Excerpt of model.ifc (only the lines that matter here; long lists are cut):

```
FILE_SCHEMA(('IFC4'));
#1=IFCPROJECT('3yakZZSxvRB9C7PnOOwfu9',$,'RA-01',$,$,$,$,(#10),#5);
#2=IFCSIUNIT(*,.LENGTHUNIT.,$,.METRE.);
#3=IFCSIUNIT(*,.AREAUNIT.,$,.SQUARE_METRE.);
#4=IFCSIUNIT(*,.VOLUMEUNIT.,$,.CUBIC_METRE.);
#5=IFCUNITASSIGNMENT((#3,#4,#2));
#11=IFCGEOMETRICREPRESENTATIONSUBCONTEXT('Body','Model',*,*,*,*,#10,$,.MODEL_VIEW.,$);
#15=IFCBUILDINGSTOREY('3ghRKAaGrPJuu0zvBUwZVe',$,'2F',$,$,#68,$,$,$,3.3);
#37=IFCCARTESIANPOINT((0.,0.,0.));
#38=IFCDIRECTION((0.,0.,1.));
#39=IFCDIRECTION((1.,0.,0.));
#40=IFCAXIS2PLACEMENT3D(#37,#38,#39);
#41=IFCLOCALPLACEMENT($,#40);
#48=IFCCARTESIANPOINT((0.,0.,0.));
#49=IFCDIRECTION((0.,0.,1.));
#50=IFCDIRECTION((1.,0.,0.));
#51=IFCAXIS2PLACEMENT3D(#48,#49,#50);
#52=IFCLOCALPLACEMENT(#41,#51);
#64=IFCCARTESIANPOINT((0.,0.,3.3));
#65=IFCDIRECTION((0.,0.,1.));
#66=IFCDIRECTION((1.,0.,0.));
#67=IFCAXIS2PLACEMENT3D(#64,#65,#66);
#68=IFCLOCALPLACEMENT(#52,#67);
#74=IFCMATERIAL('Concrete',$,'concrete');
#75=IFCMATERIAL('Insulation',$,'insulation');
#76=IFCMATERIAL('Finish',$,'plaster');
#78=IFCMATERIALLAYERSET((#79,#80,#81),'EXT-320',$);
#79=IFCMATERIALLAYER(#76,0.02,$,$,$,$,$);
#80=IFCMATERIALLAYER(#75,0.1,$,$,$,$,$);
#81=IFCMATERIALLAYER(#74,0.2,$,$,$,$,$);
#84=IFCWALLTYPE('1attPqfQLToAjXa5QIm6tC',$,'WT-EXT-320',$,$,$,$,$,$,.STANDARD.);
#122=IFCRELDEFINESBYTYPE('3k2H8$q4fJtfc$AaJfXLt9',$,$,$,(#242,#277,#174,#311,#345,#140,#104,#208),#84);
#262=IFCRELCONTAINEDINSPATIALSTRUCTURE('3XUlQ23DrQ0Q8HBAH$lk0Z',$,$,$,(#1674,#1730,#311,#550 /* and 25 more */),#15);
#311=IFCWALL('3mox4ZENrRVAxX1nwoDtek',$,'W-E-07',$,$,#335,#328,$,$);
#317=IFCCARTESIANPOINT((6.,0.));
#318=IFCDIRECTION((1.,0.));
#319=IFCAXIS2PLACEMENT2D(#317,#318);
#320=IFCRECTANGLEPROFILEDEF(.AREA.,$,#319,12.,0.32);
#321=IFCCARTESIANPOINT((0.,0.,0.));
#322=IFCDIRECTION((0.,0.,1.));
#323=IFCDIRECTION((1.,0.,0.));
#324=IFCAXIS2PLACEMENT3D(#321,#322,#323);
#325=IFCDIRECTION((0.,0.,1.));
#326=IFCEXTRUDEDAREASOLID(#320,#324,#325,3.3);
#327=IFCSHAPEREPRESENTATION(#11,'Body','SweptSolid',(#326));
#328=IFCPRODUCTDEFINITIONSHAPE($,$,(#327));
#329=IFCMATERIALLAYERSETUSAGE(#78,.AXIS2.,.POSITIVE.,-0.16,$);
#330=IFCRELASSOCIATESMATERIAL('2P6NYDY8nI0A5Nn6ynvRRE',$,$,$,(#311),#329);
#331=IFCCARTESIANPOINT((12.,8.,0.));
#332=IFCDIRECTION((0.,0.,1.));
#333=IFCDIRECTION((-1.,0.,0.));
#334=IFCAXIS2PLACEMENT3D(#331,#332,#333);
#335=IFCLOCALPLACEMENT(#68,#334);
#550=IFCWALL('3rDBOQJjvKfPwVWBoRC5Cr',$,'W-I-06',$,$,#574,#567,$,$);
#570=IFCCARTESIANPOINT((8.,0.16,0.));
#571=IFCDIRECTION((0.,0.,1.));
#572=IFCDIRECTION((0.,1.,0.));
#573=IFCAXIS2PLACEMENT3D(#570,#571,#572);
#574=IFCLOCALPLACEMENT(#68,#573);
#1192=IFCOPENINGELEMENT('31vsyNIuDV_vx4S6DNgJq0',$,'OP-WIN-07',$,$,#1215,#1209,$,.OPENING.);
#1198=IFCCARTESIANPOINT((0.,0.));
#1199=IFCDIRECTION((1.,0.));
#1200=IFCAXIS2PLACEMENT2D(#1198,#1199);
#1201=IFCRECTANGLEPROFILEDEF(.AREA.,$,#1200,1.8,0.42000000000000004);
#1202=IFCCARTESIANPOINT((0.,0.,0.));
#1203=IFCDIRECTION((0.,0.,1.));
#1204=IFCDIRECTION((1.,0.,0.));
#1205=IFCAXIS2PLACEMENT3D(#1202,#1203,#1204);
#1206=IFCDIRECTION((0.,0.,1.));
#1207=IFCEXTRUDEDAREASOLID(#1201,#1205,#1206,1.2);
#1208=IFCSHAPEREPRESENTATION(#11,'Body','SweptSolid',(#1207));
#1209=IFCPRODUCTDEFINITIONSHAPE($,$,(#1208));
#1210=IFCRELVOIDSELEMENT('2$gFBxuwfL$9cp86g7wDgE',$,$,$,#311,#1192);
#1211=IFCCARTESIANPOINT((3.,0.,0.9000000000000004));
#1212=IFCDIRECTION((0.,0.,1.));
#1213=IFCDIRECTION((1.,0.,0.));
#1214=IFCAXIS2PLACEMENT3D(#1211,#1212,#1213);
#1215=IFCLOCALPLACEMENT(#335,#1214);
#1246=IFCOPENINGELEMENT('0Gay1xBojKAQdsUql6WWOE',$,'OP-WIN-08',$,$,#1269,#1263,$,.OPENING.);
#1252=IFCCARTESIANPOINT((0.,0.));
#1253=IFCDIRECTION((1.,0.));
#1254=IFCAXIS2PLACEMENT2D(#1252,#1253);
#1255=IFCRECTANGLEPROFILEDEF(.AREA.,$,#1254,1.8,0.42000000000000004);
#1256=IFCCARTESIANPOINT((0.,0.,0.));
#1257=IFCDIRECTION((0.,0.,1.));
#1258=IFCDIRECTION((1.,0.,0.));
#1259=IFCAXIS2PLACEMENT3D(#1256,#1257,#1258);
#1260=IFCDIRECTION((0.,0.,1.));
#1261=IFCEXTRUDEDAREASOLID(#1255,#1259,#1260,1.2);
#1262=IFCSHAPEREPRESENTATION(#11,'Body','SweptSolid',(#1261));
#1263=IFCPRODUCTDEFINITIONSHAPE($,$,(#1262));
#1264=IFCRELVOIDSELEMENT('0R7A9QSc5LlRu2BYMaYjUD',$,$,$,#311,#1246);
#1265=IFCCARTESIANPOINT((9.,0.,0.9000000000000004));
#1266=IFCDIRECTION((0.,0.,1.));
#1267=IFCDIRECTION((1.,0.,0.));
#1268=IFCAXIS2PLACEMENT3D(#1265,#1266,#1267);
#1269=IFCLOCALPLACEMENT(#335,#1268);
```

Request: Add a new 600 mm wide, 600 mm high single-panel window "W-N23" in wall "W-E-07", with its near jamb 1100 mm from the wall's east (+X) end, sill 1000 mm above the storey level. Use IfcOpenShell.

```python
import numpy as np
import ifcopenshell
import ifcopenshell.api.feature
import ifcopenshell.api.geometry
import ifcopenshell.api.root
import ifcopenshell.api.spatial
import ifcopenshell.geom
import ifcopenshell.util.element
import ifcopenshell.util.placement
import ifcopenshell.util.representation
import ifcopenshell.util.shape
import ifcopenshell.util.unit

model = ifcopenshell.open("model.ifc")
unit_scale = ifcopenshell.util.unit.calculate_unit_scale(model)
settings = ifcopenshell.geom.settings()


def volume(element):
    """Net volume in cubic metres, openings subtracted."""
    shape = ifcopenshell.geom.create_shape(settings, element)
    return ifcopenshell.util.shape.get_volume(shape.geometry)


wall = model.by_id(311)
storey = ifcopenshell.util.element.get_container(wall, ifc_class="IfcBuildingStorey")
context = ifcopenshell.util.representation.get_context(model, "Model", "Body", "MODEL_VIEW")
before = volume(wall)

width, height, from_end, sill = 0.6, 0.6, 1.1, 1  # metres

# The wall runs along its own X axis, and the end named is its -X end.
wall_shape = ifcopenshell.geom.create_shape(settings, wall)
x, y, z = ifcopenshell.util.shape.get_vertices(wall_shape.geometry).T
start = x.min() + from_end
face, thickness = float(y.min()), float(y.max() - y.min())
wall_matrix = ifcopenshell.util.placement.get_local_placement(wall.ObjectPlacement)
level = ifcopenshell.util.placement.get_local_placement(storey.ObjectPlacement)[2, 3]


def in_wall(x, y):
    """Placement at x, y metres in the wall's axes, at sill height."""
    matrix = wall_matrix.copy()
    matrix[:, 3] = wall_matrix @ np.array([x / unit_scale, y / unit_scale, 0.0, 1.0])
    matrix[2, 3] = level + sill / unit_scale
    return matrix


# Opening: a box that overshoots both wall faces by 50 mm.
opening = ifcopenshell.api.root.create_entity(model, ifc_class="IfcOpeningElement", predefined_type="OPENING")
box = ifcopenshell.api.geometry.add_wall_representation(
    model, context=context, length=width, height=height, thickness=thickness + 0.1
)
ifcopenshell.api.geometry.assign_representation(model, product=opening, representation=box)
ifcopenshell.api.geometry.edit_object_placement(model, product=opening, matrix=in_wall(start, face - 0.05), is_si=False)
ifcopenshell.api.feature.add_feature(model, feature=opening, element=wall)

window = ifcopenshell.api.root.create_entity(model, ifc_class="IfcWindow", name="W-N23", predefined_type="WINDOW")
window.OverallWidth, window.OverallHeight = width / unit_scale, height / unit_scale
window.PartitioningType = "SINGLE_PANEL"
body = ifcopenshell.api.geometry.add_window_representation(
    model,
    context=context,
    overall_width=window.OverallWidth,
    overall_height=window.OverallHeight,
    partition_type="SINGLE_PANEL",
)
ifcopenshell.api.geometry.assign_representation(model, product=window, representation=body)
ifcopenshell.api.spatial.assign_container(model, products=[window], relating_structure=storey)
ifcopenshell.api.feature.add_filling(model, opening=opening, element=window)

# Centre the window in the wall's thickness.
ifcopenshell.api.geometry.edit_object_placement(model, product=window, matrix=in_wall(start, face), is_si=False)
window_shape = ifcopenshell.geom.create_shape(settings, window)
depth = ifcopenshell.util.shape.get_vertices(window_shape.geometry)[:, 1]
offset = face + thickness / 2 - (depth.min() + depth.max()) / 2
ifcopenshell.api.geometry.edit_object_placement(model, product=window, matrix=in_wall(start, offset), is_si=False)

after = volume(wall)

print(f"wall volume {before:.3f} -> {after:.3f} m3")

model.write("model_edited.ifc")
```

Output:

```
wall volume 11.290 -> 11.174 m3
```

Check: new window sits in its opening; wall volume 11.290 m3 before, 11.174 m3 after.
